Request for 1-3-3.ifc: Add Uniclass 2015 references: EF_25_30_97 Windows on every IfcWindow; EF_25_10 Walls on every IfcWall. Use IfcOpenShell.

First a look at what the model holds.

```python
import ifcopenshell

model = ifcopenshell.open("1-3-3.ifc")
print(model.schema)
print("classifications:", [c.Name for c in model.by_type("IfcClassification")])
for ifc_class in ("IfcDoor", "IfcRoof", "IfcStair", "IfcWall", "IfcWindow"):
    print(ifc_class, len(model.by_type(ifc_class)))
```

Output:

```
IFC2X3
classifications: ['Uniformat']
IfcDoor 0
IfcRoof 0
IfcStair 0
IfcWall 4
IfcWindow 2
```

```python
import ifcopenshell
import ifcopenshell.api.classification

model = ifcopenshell.open("1-3-3.ifc")

# IFC2X3 requires Source and Edition and has no link from the project to the system.
system = model.create_entity("IfcClassification", Source="NBS", Edition="2015", Name="Uniclass 2015")

codes = {
    "IfcWindow": ("EF_25_30_97", "Windows"),
    "IfcWall": ("EF_25_10", "Walls"),
}
for ifc_class, (code, name) in codes.items():
    products = model.by_type(ifc_class)
    ifcopenshell.api.classification.add_reference(
        model, products=products, classification=system, identification=code, name=name
    )
    print(code, len(products))

model.write("1-3-3_updated.ifc")
```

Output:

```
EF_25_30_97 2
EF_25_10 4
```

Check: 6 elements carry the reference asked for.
